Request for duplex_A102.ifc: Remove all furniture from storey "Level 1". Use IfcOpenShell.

First a look at what the model holds.

```python
import ifcopenshell
import ifcopenshell.util.element

model = ifcopenshell.open("duplex_A102.ifc")
print(model.schema)
storey = next(s for s in model.by_type("IfcBuildingStorey") if s.Name == "Level 1")
furniture = [e for e in ifcopenshell.util.element.get_decomposition(storey) if e.is_a("IfcFurnishingElement")]
seen = {}
for e in furniture:
    element_type = ifcopenshell.util.element.get_type(e)
    name = element_type.Name if element_type not in (None, e) else None
    seen[name] = seen.get(name, 0) + 1
for name, count in sorted(seen.items(), key=str):
    print(count, "x", name)
```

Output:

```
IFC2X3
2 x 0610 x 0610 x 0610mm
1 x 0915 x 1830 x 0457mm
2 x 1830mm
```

```python
import ifcopenshell
import ifcopenshell.api.root
import ifcopenshell.util.element

model = ifcopenshell.open("duplex_A102.ifc")

storey = next(s for s in model.by_type("IfcBuildingStorey") if s.Name == "Level 1")
furniture = [e for e in ifcopenshell.util.element.get_decomposition(storey) if e.is_a("IfcFurnishingElement")]

for e in furniture:
    ifcopenshell.api.root.remove_product(model, product=e)
print(len(furniture), "removed")

model.write("duplex_A102_edited.ifc")
```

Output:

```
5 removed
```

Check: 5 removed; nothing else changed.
